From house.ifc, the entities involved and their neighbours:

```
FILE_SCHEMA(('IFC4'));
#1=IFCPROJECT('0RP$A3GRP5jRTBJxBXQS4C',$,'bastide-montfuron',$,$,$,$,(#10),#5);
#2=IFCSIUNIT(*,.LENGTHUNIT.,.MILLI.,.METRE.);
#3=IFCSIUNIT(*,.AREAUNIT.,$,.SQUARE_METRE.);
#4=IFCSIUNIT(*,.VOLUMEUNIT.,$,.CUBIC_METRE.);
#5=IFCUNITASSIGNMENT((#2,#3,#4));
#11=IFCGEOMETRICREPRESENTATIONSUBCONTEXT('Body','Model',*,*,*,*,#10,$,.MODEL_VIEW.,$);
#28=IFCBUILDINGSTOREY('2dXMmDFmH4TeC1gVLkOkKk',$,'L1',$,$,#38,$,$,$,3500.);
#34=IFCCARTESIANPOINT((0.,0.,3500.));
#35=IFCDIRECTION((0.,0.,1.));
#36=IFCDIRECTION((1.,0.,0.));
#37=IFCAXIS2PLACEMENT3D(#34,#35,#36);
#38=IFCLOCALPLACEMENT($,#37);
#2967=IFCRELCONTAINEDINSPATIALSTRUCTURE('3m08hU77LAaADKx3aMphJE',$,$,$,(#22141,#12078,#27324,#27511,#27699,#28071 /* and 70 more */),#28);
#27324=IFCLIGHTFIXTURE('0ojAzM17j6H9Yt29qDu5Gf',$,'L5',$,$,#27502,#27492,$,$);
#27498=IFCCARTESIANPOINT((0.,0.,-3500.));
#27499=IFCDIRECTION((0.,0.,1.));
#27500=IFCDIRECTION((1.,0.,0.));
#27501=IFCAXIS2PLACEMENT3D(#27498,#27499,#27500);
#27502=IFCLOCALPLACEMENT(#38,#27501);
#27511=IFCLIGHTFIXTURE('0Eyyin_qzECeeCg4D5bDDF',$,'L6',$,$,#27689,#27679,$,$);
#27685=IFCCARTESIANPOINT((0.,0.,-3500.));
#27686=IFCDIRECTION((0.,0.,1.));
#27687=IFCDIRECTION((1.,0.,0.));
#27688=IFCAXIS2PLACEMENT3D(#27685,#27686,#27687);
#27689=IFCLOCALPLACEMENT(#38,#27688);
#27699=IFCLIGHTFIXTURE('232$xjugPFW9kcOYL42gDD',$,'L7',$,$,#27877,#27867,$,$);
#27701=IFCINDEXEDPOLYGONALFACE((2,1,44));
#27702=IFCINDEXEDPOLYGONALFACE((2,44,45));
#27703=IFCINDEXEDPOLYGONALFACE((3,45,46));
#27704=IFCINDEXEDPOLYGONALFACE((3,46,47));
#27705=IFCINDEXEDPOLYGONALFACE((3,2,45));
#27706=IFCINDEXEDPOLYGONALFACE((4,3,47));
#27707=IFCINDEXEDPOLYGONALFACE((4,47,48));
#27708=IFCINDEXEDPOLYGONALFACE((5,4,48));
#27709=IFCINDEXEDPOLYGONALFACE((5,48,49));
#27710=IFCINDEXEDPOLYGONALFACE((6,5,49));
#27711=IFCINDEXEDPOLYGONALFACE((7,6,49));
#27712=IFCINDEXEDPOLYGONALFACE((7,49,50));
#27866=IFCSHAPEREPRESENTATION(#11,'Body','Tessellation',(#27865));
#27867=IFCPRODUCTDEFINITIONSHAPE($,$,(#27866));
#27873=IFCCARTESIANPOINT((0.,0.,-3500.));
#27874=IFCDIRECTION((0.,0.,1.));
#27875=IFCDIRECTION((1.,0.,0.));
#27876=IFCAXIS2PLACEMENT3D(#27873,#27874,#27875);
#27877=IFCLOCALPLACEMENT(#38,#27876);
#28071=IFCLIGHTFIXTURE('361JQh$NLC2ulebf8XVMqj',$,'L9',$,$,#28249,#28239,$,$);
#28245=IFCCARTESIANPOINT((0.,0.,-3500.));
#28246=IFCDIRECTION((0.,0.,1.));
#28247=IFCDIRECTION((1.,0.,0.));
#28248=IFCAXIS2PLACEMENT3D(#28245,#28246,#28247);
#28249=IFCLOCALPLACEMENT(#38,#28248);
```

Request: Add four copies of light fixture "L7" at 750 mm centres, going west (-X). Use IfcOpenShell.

```python
import numpy as np
import ifcopenshell
import ifcopenshell.api.geometry
import ifcopenshell.api.root
import ifcopenshell.util.element
import ifcopenshell.util.placement
import ifcopenshell.util.unit

model = ifcopenshell.open("house.ifc")
unit_scale = ifcopenshell.util.unit.calculate_unit_scale(model)

source = model.by_guid("232$xjugPFW9kcOYL42gDD")
base = ifcopenshell.util.placement.get_local_placement(source.ObjectPlacement)
step = np.array([-1.0, 0.0, 0.0]) * 0.75 / unit_scale

for i in range(1, 5):
    copy = ifcopenshell.api.root.copy_class(model, product=source)
    copy.Representation = ifcopenshell.util.element.copy_deep(
        model, source.Representation, exclude=["IfcGeometricRepresentationContext", "IfcRepresentationMap"]
    )
    matrix = base.copy()
    matrix[:3, 3] += i * step
    print("added at", matrix[:3, 3].round(3) + 0.0)
    ifcopenshell.api.geometry.edit_object_placement(model, product=copy, matrix=matrix, is_si=False)

model.write("house_v2.ifc")
```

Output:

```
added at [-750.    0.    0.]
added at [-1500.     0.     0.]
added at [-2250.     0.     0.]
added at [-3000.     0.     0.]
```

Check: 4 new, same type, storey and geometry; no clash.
